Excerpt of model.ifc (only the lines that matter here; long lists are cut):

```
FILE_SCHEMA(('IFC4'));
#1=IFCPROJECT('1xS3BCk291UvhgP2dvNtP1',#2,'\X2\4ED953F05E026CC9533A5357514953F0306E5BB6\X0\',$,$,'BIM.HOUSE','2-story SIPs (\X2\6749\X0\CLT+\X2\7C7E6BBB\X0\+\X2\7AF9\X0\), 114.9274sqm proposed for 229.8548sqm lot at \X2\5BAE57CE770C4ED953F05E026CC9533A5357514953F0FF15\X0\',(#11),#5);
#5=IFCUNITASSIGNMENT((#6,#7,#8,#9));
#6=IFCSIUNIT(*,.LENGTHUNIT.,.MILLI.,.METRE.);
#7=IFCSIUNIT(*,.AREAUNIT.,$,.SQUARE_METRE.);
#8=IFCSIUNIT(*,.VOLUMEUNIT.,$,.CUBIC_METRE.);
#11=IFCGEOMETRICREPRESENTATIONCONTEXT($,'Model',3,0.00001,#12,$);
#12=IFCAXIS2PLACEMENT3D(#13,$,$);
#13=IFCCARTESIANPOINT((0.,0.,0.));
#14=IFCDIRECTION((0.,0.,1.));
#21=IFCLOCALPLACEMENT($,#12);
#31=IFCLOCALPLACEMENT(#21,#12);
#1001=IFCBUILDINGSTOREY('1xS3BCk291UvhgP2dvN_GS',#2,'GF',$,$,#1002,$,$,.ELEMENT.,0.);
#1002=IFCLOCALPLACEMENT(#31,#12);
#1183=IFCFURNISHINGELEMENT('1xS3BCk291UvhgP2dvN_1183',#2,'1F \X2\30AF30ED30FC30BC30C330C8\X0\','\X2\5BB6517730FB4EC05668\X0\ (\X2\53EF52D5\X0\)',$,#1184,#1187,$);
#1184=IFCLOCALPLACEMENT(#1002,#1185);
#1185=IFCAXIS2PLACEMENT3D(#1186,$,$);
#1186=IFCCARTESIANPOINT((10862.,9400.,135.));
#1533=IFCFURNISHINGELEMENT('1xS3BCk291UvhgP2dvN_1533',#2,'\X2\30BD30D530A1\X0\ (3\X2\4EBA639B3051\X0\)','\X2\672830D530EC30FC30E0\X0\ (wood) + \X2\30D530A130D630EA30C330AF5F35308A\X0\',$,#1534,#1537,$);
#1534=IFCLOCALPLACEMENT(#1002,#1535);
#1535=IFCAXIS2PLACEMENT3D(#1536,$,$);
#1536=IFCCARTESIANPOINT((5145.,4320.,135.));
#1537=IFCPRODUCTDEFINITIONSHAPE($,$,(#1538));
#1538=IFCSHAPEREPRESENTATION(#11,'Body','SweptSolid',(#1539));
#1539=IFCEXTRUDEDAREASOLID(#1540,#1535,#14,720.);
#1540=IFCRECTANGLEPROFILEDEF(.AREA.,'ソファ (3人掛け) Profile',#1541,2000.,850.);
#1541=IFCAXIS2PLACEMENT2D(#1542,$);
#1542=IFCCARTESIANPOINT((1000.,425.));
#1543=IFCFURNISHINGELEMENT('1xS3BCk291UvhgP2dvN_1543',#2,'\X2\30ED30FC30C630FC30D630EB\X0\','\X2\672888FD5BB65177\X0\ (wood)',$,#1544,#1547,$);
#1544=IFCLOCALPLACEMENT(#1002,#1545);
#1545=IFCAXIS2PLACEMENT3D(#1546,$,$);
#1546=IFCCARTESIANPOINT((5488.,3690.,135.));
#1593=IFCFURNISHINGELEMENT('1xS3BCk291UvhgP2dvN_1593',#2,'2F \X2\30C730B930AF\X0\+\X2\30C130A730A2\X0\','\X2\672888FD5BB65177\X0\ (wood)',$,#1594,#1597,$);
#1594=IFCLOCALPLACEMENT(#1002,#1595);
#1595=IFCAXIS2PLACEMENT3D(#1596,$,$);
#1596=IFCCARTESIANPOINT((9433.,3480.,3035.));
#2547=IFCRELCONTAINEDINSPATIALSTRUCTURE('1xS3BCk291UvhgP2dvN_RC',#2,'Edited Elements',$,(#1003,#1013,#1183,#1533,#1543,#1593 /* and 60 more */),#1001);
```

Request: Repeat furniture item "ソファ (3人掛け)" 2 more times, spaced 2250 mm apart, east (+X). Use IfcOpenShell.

```python
import numpy as np
import ifcopenshell
import ifcopenshell.api.geometry
import ifcopenshell.api.root
import ifcopenshell.util.element
import ifcopenshell.util.placement

model = ifcopenshell.open("model.ifc")


def reuse_history(source, copy):
    """copy_class also copies each property set's owner history, people and application; keep the originals."""
    for rel in copy.IsDefinedBy:
        if rel.is_a("IfcRelDefinesByProperties") and (history := rel.RelatingPropertyDefinition.OwnerHistory):
            rel.RelatingPropertyDefinition.OwnerHistory = source.OwnerHistory
            ifcopenshell.util.element.remove_deep2(model, history)


source = model.by_guid("1xS3BCk291UvhgP2dvN_1533")
base = ifcopenshell.util.placement.get_local_placement(source.ObjectPlacement)
step = np.array([1.0, 0.0, 0.0]) * 2250.0

for i in range(1, 3):
    copy = ifcopenshell.api.root.copy_class(model, product=source)
    copy.Representation = ifcopenshell.util.element.copy_deep(
        model, source.Representation, exclude=["IfcGeometricRepresentationContext", "IfcRepresentationMap"]
    )
    reuse_history(source, copy)
    matrix = base.copy()
    matrix[:3, 3] += i * step
    print("added at", matrix[:3, 3].round(3) + 0.0)
    ifcopenshell.api.geometry.edit_object_placement(model, product=copy, matrix=matrix, is_si=False)

model.write("model_v2.ifc")
```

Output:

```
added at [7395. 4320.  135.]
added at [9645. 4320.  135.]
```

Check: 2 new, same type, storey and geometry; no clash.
